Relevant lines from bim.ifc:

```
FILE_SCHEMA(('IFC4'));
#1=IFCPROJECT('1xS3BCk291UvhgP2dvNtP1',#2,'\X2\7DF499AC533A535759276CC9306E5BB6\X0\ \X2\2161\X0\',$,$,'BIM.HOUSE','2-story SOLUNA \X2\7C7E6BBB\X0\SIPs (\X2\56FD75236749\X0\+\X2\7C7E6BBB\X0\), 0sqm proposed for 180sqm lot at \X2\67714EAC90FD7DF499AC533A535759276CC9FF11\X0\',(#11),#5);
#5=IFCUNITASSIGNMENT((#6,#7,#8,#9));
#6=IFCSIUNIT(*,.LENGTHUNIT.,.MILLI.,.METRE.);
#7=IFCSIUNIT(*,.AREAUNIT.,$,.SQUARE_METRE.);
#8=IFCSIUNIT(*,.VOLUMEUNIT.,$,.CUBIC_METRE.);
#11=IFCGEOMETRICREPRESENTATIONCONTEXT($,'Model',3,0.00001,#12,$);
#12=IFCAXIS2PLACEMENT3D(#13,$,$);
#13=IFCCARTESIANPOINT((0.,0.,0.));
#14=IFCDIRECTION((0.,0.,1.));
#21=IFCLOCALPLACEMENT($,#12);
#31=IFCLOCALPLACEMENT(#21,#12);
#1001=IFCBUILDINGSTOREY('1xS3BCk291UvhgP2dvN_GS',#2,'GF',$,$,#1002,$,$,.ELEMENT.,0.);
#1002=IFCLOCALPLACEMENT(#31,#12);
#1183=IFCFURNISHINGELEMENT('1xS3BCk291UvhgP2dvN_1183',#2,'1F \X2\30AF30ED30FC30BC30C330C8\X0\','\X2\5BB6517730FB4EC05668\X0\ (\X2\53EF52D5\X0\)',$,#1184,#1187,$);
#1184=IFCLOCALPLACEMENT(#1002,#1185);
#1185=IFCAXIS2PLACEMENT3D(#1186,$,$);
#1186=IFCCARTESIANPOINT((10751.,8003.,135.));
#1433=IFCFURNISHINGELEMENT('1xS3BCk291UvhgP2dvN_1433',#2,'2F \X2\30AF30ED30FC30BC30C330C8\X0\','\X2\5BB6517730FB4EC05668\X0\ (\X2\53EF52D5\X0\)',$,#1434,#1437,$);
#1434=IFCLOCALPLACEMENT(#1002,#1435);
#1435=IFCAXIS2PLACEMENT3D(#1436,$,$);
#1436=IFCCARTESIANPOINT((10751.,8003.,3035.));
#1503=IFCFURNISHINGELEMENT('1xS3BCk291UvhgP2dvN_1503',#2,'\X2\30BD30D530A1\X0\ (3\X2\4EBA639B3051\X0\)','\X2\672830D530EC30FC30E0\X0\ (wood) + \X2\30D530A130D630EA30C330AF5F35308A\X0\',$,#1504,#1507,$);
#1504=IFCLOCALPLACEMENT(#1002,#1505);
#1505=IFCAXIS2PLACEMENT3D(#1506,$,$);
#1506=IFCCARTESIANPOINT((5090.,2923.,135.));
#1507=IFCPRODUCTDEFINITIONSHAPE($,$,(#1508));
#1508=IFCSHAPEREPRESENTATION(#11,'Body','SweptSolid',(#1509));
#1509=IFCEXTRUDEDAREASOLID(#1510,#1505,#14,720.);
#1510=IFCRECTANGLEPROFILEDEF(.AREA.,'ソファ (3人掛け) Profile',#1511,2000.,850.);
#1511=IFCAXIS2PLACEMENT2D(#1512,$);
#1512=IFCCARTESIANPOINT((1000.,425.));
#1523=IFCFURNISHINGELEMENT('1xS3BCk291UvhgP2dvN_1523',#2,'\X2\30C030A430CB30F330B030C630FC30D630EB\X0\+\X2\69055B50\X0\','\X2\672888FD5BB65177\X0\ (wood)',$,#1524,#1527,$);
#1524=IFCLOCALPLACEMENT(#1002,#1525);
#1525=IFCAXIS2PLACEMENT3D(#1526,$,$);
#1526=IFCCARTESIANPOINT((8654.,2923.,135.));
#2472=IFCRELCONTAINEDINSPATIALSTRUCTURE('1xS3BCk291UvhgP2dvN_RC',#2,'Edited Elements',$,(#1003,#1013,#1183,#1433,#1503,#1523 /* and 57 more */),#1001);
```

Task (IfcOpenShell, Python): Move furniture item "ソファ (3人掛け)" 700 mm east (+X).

```python
import ifcopenshell
import ifcopenshell.api.geometry
import ifcopenshell.util.placement
import ifcopenshell.util.unit

model = ifcopenshell.open("bim.ifc")
unit_scale = ifcopenshell.util.unit.calculate_unit_scale(model)

item = model.by_guid("1xS3BCk291UvhgP2dvN_1503")
matrix = ifcopenshell.util.placement.get_local_placement(item.ObjectPlacement)
matrix[0, 3] += 0.7 / unit_scale
ifcopenshell.api.geometry.edit_object_placement(model, product=item, matrix=matrix, is_si=False)

print(ifcopenshell.util.placement.get_local_placement(item.ObjectPlacement).round(3) + 0.0)

model.write("bim_edited.ifc")
```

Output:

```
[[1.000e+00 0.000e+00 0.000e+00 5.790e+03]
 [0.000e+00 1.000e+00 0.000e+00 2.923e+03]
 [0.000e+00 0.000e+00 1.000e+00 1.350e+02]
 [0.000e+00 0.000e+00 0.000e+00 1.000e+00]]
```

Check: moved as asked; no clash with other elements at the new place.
